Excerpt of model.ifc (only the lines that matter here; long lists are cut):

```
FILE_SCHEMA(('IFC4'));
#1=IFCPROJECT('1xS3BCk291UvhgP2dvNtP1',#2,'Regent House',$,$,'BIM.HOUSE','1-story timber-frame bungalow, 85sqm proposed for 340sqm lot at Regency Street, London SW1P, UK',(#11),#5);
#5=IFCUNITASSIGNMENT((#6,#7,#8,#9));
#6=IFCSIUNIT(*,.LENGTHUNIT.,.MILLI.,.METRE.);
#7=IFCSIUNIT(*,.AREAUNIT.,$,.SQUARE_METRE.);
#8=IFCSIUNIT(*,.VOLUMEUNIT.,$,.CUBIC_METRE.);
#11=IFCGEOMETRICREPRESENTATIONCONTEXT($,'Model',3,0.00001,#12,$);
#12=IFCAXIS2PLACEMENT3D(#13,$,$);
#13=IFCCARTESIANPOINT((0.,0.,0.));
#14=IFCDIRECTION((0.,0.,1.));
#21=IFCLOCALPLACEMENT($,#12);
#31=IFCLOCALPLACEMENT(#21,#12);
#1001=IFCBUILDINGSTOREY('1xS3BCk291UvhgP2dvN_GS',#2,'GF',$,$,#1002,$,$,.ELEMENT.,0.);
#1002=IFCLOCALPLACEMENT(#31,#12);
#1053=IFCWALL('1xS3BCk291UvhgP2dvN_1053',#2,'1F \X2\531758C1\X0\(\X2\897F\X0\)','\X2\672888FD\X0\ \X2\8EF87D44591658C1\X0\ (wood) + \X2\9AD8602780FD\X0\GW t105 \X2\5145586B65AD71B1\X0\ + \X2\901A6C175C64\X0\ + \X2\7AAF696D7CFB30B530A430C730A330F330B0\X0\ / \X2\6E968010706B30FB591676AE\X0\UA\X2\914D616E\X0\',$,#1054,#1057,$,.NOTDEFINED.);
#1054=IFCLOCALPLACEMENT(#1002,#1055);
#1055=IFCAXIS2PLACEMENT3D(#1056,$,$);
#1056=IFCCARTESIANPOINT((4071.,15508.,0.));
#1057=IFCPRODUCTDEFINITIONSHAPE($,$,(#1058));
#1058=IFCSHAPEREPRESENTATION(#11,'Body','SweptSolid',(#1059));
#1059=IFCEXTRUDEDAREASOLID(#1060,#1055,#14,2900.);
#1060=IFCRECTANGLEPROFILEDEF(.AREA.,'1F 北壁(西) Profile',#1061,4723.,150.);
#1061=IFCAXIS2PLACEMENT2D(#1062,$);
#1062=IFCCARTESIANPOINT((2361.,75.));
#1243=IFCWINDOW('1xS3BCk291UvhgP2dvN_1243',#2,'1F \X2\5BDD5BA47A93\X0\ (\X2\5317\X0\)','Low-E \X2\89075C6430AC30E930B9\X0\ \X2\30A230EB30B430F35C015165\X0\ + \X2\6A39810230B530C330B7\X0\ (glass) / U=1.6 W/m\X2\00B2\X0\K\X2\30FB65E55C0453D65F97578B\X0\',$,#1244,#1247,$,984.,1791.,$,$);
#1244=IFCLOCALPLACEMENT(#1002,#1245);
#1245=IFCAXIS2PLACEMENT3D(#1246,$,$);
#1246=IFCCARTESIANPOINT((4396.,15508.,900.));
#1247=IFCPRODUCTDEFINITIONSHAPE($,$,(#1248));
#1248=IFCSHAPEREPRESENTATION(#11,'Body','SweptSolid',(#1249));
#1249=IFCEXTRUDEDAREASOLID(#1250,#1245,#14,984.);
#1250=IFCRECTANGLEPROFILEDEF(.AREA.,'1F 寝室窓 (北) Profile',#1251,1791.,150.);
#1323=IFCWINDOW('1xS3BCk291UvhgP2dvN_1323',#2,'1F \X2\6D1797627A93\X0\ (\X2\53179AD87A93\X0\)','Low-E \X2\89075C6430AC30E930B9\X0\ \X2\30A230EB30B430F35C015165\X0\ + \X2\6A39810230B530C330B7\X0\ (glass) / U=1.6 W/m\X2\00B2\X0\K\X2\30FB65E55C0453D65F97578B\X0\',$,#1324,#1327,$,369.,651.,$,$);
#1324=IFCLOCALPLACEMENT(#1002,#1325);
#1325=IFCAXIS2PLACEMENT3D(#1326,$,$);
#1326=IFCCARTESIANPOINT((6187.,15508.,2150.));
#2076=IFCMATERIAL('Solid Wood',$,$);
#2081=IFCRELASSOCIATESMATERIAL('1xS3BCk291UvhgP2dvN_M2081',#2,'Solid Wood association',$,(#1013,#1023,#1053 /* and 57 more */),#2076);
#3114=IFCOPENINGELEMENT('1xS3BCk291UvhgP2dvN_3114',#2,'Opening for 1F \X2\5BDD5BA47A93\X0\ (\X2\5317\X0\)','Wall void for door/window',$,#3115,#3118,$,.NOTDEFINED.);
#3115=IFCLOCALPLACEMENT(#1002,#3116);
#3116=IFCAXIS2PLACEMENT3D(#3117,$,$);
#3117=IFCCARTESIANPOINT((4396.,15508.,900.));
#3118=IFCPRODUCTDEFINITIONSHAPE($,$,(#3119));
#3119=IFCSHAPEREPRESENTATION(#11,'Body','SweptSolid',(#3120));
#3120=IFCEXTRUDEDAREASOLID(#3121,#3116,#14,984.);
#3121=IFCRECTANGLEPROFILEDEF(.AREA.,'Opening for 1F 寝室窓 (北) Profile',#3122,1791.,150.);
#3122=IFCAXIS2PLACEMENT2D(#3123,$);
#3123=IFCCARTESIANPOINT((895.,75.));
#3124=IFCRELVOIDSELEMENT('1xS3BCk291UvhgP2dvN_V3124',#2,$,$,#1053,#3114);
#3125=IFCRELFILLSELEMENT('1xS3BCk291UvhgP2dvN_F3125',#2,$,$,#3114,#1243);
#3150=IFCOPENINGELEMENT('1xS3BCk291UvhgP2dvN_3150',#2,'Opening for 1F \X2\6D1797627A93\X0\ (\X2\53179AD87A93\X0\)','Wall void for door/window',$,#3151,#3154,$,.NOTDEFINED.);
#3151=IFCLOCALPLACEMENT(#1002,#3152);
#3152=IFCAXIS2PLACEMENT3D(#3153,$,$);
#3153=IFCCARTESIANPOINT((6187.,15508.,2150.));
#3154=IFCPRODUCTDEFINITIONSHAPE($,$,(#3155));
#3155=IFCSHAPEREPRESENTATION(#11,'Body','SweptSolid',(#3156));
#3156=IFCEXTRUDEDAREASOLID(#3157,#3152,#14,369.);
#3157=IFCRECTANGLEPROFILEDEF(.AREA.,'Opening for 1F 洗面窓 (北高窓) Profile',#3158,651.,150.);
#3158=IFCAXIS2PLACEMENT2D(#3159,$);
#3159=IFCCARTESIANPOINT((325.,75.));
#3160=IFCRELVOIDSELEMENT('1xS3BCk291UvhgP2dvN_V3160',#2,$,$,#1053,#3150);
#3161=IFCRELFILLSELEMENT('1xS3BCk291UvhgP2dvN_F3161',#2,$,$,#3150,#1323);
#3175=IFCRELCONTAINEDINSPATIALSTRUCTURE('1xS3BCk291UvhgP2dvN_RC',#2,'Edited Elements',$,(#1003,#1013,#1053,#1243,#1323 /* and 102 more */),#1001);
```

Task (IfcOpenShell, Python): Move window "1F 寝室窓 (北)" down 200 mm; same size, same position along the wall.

```python
import numpy as np
import ifcopenshell
import ifcopenshell.api.geometry
import ifcopenshell.util.placement
import ifcopenshell.util.unit

model = ifcopenshell.open("model.ifc")
unit_scale = ifcopenshell.util.unit.calculate_unit_scale(model)

window = model.by_id(1243)
opening = window.FillsVoids[0].RelatingOpeningElement
dz = -0.2 / unit_scale

shift = np.array([0.0, 0.0, dz])
# The window is not placed relative to its opening, so move both.
for product in (opening, window):
    matrix = ifcopenshell.util.placement.get_local_placement(product.ObjectPlacement)
    matrix[:3, 3] += shift
    ifcopenshell.api.geometry.edit_object_placement(model, product=product, matrix=matrix, is_si=False)

print(f"moved by {dz * unit_scale:+.3f} m")

model.write("model-out.ifc")
```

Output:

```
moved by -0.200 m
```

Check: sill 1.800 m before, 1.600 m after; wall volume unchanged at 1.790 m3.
